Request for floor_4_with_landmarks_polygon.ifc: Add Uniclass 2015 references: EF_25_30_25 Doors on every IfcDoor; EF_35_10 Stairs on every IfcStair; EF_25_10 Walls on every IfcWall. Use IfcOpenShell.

First a look at what the model holds.

```python
import ifcopenshell

model = ifcopenshell.open("floor_4_with_landmarks_polygon.ifc")
print(model.schema)
print("classifications:", [c.Name for c in model.by_type("IfcClassification")])
for ifc_class in ("IfcDoor", "IfcRoof", "IfcStair", "IfcWall", "IfcWindow"):
    print(ifc_class, len(model.by_type(ifc_class)))
```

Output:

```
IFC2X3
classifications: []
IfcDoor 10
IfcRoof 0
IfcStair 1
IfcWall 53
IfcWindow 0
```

```python
import ifcopenshell
import ifcopenshell.api.classification

model = ifcopenshell.open("floor_4_with_landmarks_polygon.ifc")

# IFC2X3 requires Source and Edition and has no link from the project to the system.
system = model.create_entity("IfcClassification", Source="NBS", Edition="2015", Name="Uniclass 2015")

codes = {
    "IfcDoor": ("EF_25_30_25", "Doors"),
    "IfcStair": ("EF_35_10", "Stairs"),
    "IfcWall": ("EF_25_10", "Walls"),
}
for ifc_class, (code, name) in codes.items():
    products = model.by_type(ifc_class)
    ifcopenshell.api.classification.add_reference(
        model, products=products, classification=system, identification=code, name=name
    )
    print(code, len(products))

model.write("floor_4_with_landmarks_polygon-out.ifc")
```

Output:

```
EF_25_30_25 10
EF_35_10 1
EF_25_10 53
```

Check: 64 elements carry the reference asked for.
